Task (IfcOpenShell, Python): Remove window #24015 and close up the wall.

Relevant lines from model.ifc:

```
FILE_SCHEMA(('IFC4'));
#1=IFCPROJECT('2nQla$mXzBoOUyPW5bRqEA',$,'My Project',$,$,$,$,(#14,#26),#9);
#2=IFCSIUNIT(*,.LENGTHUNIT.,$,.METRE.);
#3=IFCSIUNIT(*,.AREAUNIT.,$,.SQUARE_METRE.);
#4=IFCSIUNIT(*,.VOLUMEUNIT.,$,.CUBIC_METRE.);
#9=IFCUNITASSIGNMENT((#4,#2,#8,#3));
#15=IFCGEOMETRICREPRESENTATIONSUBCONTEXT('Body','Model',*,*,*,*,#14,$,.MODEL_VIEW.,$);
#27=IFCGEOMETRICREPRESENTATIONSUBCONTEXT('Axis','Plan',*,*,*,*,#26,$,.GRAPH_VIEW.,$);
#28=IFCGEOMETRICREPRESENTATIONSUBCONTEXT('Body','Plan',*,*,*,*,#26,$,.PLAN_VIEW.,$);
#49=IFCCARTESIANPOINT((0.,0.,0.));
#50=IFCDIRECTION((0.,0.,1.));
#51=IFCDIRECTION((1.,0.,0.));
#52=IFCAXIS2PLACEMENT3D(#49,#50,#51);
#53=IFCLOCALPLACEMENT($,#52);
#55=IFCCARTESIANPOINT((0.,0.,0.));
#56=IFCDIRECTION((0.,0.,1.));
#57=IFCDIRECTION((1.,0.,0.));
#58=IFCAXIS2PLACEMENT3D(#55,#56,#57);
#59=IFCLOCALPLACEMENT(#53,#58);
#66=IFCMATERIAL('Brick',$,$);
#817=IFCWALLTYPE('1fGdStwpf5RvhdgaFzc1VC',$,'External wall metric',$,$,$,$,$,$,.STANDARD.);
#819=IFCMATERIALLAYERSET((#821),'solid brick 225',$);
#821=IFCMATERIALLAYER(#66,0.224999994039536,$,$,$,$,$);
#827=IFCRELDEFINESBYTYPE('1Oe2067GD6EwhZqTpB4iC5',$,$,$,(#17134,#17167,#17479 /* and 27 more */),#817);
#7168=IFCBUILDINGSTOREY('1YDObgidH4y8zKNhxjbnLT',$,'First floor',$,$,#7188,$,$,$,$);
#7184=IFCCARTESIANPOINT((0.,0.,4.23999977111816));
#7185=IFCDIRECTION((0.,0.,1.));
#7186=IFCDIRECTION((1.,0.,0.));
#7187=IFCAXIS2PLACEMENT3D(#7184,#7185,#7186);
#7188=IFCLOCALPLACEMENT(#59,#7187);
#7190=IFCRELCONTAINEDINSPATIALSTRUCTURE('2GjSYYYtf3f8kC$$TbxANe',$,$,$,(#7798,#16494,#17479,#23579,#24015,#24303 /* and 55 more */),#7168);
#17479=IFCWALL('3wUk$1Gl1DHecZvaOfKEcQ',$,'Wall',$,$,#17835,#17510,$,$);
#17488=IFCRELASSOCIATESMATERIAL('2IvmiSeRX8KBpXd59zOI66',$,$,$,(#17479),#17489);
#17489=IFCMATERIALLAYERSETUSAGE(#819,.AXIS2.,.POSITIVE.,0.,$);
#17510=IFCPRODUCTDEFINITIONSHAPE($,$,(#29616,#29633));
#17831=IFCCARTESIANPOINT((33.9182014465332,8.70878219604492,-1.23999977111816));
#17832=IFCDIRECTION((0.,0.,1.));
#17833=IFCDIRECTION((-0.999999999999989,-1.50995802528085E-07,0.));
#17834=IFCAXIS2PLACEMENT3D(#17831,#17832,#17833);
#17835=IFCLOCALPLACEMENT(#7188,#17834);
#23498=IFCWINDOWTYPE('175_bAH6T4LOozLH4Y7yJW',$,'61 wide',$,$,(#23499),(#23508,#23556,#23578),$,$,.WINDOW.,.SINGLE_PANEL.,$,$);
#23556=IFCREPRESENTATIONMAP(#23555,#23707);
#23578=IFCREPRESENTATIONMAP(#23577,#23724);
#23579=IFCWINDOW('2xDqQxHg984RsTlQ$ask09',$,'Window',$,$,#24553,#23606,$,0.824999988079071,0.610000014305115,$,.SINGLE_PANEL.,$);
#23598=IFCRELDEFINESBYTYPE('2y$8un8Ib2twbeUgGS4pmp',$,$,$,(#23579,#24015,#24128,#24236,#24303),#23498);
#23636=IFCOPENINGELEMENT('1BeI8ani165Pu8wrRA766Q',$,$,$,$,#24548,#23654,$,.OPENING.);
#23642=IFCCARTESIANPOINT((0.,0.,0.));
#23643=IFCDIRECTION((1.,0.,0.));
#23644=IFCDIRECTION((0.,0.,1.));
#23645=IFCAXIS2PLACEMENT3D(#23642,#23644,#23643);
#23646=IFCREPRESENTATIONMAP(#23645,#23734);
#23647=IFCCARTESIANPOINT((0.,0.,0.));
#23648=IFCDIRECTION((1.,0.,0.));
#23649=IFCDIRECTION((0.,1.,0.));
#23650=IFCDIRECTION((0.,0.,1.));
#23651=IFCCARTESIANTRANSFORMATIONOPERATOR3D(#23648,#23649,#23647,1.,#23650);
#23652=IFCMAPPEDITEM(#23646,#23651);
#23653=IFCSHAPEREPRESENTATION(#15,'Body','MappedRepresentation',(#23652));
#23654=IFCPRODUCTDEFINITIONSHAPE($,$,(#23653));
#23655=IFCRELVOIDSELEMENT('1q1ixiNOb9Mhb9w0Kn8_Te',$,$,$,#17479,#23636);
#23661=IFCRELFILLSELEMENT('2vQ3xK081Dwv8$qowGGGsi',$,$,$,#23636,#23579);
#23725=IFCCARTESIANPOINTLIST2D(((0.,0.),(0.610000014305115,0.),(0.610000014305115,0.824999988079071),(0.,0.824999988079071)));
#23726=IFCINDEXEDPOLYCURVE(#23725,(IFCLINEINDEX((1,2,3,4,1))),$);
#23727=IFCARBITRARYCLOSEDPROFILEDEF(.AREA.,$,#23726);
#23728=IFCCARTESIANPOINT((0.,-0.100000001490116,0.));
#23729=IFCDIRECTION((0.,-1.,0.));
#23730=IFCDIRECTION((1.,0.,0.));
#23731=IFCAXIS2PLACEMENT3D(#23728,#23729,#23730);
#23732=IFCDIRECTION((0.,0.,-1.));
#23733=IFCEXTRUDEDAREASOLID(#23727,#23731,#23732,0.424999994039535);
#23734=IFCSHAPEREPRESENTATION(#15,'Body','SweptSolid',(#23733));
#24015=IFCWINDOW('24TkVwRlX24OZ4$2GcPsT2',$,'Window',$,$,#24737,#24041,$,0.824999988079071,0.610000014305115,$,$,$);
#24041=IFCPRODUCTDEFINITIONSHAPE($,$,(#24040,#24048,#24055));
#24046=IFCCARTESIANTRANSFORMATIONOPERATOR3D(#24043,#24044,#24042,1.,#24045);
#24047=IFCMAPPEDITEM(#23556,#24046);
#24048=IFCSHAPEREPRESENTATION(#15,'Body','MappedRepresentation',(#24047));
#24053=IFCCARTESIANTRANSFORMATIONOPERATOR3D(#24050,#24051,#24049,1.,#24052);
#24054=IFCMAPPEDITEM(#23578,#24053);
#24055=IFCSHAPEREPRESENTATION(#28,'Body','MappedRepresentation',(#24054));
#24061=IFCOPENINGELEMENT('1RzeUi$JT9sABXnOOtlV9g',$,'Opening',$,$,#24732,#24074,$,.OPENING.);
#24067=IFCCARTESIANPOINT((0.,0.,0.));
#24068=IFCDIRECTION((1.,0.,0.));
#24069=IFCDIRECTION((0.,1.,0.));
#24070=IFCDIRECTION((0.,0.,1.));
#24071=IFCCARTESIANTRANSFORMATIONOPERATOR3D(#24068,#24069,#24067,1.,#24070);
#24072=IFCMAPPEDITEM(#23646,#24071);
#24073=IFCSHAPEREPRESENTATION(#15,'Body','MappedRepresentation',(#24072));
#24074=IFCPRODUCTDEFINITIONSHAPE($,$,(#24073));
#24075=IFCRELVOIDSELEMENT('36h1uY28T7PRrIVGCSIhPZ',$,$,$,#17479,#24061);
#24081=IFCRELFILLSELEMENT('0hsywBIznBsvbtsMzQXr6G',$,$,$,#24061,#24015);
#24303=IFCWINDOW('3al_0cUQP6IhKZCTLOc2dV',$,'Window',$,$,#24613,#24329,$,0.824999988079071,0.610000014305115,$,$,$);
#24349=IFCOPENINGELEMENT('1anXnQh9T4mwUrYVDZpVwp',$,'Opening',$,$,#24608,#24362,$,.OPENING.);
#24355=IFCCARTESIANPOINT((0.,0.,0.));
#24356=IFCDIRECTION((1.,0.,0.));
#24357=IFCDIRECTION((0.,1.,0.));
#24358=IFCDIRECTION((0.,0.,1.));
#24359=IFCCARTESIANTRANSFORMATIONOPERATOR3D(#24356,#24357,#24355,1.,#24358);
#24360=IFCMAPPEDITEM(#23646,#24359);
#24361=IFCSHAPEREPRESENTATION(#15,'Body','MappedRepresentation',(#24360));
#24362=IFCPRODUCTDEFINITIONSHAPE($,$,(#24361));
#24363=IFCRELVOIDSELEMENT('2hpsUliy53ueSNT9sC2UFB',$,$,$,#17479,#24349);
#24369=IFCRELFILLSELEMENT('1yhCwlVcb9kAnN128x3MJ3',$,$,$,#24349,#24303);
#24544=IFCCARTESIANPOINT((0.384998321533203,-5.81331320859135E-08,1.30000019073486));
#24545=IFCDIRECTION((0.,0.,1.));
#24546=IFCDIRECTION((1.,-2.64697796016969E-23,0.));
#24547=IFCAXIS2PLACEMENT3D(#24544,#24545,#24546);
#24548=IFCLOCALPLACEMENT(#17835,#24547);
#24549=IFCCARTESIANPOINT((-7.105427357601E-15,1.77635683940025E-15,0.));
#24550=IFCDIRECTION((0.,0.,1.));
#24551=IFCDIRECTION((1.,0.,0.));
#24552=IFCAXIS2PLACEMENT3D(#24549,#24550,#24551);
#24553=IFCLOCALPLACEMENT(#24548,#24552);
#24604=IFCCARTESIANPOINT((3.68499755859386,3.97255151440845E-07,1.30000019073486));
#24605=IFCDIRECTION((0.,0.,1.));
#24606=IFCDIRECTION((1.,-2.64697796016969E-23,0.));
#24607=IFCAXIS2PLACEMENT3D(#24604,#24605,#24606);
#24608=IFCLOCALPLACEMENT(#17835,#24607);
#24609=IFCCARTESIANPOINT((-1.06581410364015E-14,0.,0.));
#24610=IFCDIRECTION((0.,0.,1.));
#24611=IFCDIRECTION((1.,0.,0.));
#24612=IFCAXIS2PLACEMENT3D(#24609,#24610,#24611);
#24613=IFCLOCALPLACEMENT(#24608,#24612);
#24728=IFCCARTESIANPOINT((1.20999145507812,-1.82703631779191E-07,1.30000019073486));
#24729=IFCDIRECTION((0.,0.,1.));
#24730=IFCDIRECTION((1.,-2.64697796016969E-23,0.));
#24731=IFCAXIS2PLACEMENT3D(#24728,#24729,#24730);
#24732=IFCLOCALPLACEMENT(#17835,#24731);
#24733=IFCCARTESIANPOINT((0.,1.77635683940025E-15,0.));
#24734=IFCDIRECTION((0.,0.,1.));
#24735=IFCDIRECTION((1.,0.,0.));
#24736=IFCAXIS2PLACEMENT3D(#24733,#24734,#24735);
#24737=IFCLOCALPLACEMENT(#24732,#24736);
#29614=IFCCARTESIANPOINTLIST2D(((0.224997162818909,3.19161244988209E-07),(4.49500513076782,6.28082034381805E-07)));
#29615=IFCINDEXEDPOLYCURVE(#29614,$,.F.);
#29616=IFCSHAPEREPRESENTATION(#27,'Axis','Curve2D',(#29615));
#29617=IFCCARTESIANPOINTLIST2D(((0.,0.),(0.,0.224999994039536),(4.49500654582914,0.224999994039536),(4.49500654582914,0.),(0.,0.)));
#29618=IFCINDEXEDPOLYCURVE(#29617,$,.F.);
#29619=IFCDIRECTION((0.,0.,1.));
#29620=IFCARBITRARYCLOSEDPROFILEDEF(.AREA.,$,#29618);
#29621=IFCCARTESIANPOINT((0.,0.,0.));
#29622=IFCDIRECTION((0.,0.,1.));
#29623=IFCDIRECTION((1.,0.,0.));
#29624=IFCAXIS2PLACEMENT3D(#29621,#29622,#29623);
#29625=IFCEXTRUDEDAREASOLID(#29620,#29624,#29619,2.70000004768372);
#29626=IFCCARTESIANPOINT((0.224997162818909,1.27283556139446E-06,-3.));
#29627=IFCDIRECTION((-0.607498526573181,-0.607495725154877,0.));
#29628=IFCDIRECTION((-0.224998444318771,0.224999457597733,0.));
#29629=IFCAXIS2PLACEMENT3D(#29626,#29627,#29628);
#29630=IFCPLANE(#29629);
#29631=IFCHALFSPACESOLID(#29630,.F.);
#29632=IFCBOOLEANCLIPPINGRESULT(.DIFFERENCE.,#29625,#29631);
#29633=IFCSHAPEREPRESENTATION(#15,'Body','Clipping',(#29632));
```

```python
import ifcopenshell
import ifcopenshell.api.feature
import ifcopenshell.api.root
import ifcopenshell.geom
import ifcopenshell.util.shape

model = ifcopenshell.open("model.ifc")
settings = ifcopenshell.geom.settings()


def volume(element):
    """Net volume in cubic metres, openings subtracted."""
    shape = ifcopenshell.geom.create_shape(settings, element)
    return ifcopenshell.util.shape.get_volume(shape.geometry)


window = model.by_guid("24TkVwRlX24OZ4$2GcPsT2")
opening = window.FillsVoids[0].RelatingOpeningElement
wall = opening.VoidsElements[0].RelatingBuildingElement
before = volume(wall)

ifcopenshell.api.root.remove_product(model, product=window)
ifcopenshell.api.feature.remove_feature(model, feature=opening)

after = volume(wall)

print(f"wall volume {before:.3f} -> {after:.3f} m3")

model.write("model_rev.ifc")
```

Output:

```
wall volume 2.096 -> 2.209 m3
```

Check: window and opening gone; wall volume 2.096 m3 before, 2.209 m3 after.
